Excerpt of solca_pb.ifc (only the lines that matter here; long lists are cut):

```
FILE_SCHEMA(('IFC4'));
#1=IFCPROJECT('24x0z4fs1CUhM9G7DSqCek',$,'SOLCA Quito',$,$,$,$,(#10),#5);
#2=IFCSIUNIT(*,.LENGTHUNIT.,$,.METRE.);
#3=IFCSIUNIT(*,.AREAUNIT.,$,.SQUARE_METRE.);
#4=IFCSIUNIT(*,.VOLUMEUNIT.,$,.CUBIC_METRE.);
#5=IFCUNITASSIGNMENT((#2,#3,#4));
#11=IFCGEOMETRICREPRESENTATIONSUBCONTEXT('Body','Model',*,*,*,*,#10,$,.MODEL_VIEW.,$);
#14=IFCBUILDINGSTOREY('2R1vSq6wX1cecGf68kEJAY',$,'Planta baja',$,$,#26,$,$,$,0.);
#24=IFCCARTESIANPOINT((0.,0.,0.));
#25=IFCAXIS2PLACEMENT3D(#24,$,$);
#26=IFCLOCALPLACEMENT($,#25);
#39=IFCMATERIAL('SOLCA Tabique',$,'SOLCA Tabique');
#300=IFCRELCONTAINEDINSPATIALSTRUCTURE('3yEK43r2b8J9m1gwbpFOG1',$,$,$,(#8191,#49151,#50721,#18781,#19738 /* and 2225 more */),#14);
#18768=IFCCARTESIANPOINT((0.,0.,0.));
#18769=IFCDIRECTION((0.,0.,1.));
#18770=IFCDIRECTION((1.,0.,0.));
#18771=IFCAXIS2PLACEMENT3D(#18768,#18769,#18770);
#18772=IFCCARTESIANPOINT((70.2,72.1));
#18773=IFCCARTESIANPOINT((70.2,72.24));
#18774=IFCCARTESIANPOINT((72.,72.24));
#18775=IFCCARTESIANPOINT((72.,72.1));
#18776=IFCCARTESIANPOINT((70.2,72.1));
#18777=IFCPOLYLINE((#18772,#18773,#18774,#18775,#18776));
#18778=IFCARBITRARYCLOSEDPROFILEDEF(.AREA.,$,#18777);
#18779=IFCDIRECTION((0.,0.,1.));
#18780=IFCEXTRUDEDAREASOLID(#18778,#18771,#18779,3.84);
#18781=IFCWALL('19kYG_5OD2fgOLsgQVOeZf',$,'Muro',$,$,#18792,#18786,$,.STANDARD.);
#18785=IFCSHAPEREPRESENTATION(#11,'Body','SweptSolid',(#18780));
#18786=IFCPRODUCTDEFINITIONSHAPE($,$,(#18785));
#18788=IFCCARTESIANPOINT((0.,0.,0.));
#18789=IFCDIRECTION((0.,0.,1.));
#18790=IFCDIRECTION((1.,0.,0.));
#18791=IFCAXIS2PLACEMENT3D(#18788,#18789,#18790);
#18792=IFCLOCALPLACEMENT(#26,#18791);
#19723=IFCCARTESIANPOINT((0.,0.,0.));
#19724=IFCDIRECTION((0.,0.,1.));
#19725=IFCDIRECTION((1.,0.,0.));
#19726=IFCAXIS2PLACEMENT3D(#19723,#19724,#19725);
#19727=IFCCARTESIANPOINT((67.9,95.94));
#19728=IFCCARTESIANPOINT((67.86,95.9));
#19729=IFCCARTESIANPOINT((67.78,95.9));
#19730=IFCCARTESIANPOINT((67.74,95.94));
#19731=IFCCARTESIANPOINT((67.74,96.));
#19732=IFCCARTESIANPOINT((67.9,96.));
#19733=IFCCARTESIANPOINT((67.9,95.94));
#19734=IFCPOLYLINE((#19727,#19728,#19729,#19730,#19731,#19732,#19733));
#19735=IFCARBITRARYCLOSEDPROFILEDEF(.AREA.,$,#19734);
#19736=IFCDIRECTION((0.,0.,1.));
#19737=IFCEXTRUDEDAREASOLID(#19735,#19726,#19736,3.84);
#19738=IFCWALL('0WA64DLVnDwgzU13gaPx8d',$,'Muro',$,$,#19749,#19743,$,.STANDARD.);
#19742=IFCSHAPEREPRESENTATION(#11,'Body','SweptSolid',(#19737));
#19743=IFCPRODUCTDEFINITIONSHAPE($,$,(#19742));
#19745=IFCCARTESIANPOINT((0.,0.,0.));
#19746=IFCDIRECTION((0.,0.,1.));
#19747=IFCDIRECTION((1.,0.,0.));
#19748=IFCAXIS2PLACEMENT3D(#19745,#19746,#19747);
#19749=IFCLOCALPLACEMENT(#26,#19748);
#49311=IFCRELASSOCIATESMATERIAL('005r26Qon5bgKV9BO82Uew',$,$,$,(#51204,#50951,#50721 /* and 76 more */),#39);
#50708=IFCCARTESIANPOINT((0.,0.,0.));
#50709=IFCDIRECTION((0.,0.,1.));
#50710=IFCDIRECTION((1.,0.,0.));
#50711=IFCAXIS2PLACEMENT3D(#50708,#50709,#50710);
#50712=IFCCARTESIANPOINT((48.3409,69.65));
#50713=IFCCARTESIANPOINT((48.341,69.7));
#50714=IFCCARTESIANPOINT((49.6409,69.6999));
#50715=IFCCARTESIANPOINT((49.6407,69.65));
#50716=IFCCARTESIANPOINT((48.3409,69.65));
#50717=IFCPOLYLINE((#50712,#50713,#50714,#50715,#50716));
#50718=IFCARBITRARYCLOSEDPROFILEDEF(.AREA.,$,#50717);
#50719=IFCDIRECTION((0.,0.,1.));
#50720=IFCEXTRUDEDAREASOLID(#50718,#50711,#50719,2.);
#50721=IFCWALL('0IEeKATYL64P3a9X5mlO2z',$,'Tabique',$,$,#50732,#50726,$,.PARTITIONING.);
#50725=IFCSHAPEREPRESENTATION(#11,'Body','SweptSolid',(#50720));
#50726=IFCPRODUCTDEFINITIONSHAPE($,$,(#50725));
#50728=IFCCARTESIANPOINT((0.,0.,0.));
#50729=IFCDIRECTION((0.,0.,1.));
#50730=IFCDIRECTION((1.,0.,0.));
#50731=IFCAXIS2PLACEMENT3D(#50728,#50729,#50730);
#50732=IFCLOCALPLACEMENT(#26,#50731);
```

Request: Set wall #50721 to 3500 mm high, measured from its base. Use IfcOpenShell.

```python
import ifcopenshell
import ifcopenshell.geom
import ifcopenshell.util.representation
import ifcopenshell.util.shape

model = ifcopenshell.open("solca_pb.ifc")
settings = ifcopenshell.geom.settings()


def volume(element):
    """Net volume in cubic metres, openings subtracted."""
    shape = ifcopenshell.geom.create_shape(settings, element)
    return ifcopenshell.util.shape.get_volume(shape.geometry)


wall = model.by_guid("0IEeKATYL64P3a9X5mlO2z")
before = volume(wall)

body = ifcopenshell.util.representation.get_representation(wall, "Model", "Body")
solid = body.Items[0]
old_height = solid.Depth
solid.Depth = 3.5
after = volume(wall)

print(f"height {old_height:g} -> {solid.Depth:g}, volume {before:.3f} -> {after:.3f} m3")

model.write("solca_pb_v2.ifc")
```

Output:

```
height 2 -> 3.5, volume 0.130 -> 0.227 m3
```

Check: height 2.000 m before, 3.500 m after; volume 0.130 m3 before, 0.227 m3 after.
